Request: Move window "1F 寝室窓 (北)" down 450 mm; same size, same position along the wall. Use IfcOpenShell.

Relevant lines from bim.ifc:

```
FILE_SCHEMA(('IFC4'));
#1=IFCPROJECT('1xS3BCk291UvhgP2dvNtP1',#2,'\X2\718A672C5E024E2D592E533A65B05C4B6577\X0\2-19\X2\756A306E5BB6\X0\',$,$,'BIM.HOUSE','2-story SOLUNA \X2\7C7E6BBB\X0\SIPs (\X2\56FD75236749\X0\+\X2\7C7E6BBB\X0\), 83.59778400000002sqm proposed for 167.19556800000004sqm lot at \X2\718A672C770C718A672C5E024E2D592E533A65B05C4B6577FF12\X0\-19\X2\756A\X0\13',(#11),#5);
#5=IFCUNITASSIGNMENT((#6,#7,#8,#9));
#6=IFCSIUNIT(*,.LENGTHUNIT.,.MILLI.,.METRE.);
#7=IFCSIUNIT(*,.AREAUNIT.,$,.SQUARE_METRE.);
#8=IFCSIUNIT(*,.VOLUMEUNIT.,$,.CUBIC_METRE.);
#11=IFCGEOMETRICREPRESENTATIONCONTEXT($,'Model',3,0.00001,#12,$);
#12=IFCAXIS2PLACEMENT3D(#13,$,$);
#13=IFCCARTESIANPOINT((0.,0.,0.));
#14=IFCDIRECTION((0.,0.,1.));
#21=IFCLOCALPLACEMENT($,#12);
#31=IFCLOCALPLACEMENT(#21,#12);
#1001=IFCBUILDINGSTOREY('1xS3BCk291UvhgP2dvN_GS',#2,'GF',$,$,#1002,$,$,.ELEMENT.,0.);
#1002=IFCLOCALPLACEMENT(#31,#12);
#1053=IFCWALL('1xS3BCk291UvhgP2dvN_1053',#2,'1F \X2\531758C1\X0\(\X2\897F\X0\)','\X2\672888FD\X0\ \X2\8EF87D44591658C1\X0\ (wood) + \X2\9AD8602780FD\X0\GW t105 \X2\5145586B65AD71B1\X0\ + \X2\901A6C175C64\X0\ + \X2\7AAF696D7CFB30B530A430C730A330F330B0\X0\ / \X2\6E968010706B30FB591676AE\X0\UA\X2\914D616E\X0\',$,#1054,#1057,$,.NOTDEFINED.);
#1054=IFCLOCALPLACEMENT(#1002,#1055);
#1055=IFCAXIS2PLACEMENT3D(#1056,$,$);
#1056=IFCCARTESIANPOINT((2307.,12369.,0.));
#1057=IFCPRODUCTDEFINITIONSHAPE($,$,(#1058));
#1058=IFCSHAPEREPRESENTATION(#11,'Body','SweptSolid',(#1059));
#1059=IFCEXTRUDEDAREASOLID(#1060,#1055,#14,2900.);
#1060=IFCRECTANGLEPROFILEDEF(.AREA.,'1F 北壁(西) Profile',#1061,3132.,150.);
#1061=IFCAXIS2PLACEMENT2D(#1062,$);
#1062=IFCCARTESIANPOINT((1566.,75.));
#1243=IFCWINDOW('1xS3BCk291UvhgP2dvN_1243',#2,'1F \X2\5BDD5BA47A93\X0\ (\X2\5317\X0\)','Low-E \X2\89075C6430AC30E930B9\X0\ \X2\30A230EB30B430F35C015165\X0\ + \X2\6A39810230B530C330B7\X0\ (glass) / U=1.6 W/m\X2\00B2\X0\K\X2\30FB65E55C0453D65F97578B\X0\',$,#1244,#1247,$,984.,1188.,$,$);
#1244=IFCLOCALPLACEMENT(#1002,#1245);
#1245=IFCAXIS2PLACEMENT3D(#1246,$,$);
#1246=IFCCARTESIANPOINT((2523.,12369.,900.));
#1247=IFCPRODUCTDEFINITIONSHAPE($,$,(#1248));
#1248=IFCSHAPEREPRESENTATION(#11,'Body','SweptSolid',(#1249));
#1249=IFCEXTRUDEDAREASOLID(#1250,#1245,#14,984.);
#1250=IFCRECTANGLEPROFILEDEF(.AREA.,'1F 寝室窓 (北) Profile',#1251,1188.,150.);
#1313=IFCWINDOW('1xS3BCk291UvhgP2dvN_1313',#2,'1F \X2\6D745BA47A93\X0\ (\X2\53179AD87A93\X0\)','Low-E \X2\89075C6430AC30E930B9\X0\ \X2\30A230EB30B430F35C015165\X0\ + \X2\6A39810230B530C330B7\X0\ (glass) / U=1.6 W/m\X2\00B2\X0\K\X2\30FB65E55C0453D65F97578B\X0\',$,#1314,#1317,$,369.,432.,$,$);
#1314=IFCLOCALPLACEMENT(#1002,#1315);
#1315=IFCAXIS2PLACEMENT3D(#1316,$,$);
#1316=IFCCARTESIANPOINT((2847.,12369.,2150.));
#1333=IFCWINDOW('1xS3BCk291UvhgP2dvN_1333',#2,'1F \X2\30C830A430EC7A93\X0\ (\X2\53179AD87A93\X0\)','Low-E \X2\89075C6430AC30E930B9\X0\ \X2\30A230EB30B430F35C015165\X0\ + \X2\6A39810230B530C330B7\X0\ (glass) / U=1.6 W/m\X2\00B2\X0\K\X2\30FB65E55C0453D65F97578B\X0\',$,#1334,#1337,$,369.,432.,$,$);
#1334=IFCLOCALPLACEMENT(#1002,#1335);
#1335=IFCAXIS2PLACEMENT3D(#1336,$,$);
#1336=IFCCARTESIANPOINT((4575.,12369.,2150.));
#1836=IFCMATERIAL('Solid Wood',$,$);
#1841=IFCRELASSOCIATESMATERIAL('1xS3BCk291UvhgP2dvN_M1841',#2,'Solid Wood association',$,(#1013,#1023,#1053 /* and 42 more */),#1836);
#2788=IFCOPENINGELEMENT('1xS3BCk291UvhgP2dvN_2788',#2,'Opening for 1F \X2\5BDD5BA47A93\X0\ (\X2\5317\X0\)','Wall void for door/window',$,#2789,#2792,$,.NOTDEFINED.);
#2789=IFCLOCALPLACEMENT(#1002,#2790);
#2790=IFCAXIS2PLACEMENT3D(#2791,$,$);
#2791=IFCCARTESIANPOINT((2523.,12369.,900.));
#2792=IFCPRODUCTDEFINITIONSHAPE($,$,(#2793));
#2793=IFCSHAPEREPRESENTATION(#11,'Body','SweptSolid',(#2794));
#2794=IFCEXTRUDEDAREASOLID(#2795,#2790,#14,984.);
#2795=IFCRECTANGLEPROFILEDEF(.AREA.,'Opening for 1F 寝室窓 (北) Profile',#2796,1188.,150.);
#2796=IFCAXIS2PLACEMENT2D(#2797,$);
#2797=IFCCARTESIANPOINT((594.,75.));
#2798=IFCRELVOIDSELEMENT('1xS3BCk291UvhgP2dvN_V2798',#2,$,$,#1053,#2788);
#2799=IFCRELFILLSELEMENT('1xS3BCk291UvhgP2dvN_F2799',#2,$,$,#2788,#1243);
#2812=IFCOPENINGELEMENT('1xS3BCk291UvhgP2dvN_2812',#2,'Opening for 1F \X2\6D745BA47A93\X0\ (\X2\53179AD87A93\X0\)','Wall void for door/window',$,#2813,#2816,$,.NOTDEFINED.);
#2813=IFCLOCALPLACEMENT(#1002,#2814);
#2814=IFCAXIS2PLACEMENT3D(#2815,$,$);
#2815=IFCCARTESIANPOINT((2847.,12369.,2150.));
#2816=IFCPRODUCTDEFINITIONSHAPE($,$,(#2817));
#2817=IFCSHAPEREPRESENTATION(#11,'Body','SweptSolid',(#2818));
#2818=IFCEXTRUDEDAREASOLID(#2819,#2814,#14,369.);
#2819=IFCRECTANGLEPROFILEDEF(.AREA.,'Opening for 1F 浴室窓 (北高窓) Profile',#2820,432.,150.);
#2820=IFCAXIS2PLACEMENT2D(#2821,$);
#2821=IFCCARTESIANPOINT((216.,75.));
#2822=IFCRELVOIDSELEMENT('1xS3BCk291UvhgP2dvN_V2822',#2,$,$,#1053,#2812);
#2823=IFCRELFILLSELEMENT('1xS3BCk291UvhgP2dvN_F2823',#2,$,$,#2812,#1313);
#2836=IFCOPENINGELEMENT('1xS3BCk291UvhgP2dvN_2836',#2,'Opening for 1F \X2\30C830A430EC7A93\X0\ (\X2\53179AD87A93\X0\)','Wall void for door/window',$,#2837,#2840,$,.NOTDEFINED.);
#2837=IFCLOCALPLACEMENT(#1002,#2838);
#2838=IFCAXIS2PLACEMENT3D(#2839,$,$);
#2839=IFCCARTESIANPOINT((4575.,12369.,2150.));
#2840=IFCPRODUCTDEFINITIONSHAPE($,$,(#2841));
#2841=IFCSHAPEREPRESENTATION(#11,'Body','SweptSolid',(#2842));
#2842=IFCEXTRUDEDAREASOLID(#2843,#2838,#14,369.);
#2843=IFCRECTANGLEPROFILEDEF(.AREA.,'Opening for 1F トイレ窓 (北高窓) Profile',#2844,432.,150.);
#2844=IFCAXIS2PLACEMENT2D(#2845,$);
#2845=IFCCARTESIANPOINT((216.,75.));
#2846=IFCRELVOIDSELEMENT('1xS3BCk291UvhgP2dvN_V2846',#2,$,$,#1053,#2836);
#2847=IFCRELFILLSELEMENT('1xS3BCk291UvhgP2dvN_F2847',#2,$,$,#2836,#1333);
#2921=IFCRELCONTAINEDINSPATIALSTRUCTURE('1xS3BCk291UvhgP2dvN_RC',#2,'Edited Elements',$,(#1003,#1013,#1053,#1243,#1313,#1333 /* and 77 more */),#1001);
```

```python
import numpy as np
import ifcopenshell
import ifcopenshell.api.geometry
import ifcopenshell.util.placement
import ifcopenshell.util.unit

model = ifcopenshell.open("bim.ifc")
unit_scale = ifcopenshell.util.unit.calculate_unit_scale(model)

window = model.by_id(1243)
opening = window.FillsVoids[0].RelatingOpeningElement
dz = -450.0

shift = np.array([0.0, 0.0, dz])
# The window is not placed relative to its opening, so move both.
for product in (opening, window):
    matrix = ifcopenshell.util.placement.get_local_placement(product.ObjectPlacement)
    matrix[:3, 3] += shift
    ifcopenshell.api.geometry.edit_object_placement(model, product=product, matrix=matrix, is_si=False)

print(f"moved by {dz * unit_scale:+.3f} m")

model.write("bim_v2.ifc")
```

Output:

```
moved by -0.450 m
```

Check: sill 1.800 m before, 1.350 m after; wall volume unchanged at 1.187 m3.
